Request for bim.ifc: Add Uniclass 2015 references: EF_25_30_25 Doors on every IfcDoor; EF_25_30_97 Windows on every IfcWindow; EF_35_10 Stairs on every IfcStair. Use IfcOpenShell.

First a look at what the model holds.

```python
import ifcopenshell

model = ifcopenshell.open("bim.ifc")
print(model.schema)
print("classifications:", [c.Name for c in model.by_type("IfcClassification")])
for ifc_class in ("IfcDoor", "IfcRoof", "IfcStair", "IfcWall", "IfcWindow"):
    print(ifc_class, len(model.by_type(ifc_class)))
```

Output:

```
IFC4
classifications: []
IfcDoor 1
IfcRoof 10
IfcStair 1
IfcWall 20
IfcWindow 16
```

```python
import ifcopenshell
import ifcopenshell.api.classification

model = ifcopenshell.open("bim.ifc")

system = ifcopenshell.api.classification.add_classification(model, classification="Uniclass 2015")

codes = {
    "IfcDoor": ("EF_25_30_25", "Doors"),
    "IfcWindow": ("EF_25_30_97", "Windows"),
    "IfcStair": ("EF_35_10", "Stairs"),
}
for ifc_class, (code, name) in codes.items():
    products = model.by_type(ifc_class)
    ifcopenshell.api.classification.add_reference(
        model, products=products, classification=system, identification=code, name=name
    )
    print(code, len(products))

model.write("bim_v2.ifc")
```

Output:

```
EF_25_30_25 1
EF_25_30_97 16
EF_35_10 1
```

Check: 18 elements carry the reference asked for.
